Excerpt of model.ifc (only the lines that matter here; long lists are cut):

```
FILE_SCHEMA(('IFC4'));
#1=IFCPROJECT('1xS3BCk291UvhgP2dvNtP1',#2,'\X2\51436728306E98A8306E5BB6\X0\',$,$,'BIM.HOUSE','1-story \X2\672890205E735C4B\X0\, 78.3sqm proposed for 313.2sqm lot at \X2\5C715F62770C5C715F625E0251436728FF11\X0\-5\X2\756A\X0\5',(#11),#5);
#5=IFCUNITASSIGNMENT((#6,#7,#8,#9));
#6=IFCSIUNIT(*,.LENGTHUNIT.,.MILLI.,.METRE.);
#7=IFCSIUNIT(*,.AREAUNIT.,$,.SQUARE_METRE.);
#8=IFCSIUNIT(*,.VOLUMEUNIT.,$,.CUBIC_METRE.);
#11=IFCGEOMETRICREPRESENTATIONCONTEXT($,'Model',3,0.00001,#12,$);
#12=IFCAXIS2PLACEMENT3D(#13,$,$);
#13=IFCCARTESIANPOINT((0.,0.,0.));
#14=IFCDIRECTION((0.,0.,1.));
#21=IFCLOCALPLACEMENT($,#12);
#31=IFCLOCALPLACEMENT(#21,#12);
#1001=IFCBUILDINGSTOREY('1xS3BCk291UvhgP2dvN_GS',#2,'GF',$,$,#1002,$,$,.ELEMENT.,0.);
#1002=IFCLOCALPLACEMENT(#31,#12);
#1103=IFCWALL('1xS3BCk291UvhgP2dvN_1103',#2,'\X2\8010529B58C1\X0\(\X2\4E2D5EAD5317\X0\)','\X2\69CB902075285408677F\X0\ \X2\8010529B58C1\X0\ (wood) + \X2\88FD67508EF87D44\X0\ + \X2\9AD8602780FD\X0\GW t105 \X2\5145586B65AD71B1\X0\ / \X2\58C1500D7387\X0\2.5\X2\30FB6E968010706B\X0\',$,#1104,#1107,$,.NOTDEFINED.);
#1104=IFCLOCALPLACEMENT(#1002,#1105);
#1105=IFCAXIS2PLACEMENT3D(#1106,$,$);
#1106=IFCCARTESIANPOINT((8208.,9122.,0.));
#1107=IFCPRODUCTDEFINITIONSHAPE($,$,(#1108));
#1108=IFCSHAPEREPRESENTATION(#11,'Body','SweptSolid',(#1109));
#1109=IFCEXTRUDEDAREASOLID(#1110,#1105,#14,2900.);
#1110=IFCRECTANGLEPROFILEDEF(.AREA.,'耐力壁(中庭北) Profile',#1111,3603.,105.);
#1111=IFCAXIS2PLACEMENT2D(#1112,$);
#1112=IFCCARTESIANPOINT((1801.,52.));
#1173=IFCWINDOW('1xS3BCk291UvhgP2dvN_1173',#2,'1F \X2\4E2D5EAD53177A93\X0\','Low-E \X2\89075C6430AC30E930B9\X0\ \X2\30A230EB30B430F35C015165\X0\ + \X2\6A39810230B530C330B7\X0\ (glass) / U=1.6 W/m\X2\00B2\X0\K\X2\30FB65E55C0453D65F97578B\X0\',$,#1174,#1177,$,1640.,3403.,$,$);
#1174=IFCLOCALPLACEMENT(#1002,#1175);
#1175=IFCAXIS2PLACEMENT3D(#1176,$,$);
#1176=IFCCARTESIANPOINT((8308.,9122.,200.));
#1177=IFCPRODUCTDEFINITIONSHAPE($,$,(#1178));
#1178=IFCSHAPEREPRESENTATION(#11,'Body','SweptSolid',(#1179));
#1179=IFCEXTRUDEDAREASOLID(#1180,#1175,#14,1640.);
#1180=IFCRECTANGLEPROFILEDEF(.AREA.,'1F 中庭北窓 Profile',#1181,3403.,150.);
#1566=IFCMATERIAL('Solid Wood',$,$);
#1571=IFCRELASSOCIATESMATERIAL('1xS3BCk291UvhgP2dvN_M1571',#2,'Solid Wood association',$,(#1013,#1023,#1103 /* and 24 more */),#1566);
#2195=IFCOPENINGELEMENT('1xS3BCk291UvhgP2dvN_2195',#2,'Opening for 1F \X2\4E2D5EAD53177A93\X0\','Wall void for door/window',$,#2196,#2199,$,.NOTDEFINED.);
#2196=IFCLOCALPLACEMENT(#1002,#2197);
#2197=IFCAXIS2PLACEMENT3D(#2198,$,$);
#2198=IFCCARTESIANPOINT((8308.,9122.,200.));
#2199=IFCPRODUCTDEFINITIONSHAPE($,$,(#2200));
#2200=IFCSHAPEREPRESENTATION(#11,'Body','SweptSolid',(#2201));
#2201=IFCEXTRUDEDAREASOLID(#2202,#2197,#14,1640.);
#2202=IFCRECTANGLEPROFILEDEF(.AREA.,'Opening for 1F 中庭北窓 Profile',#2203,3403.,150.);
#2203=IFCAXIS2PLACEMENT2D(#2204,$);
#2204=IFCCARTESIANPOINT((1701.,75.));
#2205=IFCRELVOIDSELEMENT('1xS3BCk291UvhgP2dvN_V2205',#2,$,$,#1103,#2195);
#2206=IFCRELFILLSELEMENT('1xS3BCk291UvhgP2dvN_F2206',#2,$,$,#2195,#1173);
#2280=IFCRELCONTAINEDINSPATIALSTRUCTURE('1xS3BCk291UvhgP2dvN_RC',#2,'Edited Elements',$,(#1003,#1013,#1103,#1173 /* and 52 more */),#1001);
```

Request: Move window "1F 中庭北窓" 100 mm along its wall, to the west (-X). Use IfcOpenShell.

```python
import ifcopenshell
import ifcopenshell.api.geometry
import ifcopenshell.util.placement
import ifcopenshell.util.unit

model = ifcopenshell.open("model.ifc")
unit_scale = ifcopenshell.util.unit.calculate_unit_scale(model)

window = model.by_guid("1xS3BCk291UvhgP2dvN_1173")
opening = window.FillsVoids[0].RelatingOpeningElement
wall = opening.VoidsElements[0].RelatingBuildingElement

wall_matrix = ifcopenshell.util.placement.get_local_placement(wall.ObjectPlacement)
shift = wall_matrix[:3, 0] * -0.1 / unit_scale
before = ifcopenshell.util.placement.get_local_placement(window.ObjectPlacement)[:3, 3].copy()

# The window is not placed relative to its opening, so move both.
for product in (opening, window):
    matrix = ifcopenshell.util.placement.get_local_placement(product.ObjectPlacement)
    matrix[:3, 3] += shift
    ifcopenshell.api.geometry.edit_object_placement(model, product=product, matrix=matrix, is_si=False)

after = ifcopenshell.util.placement.get_local_placement(window.ObjectPlacement)[:3, 3]
print("window moved by", (after - before).round(3) + 0.0)

model.write("model_v2.ifc")
```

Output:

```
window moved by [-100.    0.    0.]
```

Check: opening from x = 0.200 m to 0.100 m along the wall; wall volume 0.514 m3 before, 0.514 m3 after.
